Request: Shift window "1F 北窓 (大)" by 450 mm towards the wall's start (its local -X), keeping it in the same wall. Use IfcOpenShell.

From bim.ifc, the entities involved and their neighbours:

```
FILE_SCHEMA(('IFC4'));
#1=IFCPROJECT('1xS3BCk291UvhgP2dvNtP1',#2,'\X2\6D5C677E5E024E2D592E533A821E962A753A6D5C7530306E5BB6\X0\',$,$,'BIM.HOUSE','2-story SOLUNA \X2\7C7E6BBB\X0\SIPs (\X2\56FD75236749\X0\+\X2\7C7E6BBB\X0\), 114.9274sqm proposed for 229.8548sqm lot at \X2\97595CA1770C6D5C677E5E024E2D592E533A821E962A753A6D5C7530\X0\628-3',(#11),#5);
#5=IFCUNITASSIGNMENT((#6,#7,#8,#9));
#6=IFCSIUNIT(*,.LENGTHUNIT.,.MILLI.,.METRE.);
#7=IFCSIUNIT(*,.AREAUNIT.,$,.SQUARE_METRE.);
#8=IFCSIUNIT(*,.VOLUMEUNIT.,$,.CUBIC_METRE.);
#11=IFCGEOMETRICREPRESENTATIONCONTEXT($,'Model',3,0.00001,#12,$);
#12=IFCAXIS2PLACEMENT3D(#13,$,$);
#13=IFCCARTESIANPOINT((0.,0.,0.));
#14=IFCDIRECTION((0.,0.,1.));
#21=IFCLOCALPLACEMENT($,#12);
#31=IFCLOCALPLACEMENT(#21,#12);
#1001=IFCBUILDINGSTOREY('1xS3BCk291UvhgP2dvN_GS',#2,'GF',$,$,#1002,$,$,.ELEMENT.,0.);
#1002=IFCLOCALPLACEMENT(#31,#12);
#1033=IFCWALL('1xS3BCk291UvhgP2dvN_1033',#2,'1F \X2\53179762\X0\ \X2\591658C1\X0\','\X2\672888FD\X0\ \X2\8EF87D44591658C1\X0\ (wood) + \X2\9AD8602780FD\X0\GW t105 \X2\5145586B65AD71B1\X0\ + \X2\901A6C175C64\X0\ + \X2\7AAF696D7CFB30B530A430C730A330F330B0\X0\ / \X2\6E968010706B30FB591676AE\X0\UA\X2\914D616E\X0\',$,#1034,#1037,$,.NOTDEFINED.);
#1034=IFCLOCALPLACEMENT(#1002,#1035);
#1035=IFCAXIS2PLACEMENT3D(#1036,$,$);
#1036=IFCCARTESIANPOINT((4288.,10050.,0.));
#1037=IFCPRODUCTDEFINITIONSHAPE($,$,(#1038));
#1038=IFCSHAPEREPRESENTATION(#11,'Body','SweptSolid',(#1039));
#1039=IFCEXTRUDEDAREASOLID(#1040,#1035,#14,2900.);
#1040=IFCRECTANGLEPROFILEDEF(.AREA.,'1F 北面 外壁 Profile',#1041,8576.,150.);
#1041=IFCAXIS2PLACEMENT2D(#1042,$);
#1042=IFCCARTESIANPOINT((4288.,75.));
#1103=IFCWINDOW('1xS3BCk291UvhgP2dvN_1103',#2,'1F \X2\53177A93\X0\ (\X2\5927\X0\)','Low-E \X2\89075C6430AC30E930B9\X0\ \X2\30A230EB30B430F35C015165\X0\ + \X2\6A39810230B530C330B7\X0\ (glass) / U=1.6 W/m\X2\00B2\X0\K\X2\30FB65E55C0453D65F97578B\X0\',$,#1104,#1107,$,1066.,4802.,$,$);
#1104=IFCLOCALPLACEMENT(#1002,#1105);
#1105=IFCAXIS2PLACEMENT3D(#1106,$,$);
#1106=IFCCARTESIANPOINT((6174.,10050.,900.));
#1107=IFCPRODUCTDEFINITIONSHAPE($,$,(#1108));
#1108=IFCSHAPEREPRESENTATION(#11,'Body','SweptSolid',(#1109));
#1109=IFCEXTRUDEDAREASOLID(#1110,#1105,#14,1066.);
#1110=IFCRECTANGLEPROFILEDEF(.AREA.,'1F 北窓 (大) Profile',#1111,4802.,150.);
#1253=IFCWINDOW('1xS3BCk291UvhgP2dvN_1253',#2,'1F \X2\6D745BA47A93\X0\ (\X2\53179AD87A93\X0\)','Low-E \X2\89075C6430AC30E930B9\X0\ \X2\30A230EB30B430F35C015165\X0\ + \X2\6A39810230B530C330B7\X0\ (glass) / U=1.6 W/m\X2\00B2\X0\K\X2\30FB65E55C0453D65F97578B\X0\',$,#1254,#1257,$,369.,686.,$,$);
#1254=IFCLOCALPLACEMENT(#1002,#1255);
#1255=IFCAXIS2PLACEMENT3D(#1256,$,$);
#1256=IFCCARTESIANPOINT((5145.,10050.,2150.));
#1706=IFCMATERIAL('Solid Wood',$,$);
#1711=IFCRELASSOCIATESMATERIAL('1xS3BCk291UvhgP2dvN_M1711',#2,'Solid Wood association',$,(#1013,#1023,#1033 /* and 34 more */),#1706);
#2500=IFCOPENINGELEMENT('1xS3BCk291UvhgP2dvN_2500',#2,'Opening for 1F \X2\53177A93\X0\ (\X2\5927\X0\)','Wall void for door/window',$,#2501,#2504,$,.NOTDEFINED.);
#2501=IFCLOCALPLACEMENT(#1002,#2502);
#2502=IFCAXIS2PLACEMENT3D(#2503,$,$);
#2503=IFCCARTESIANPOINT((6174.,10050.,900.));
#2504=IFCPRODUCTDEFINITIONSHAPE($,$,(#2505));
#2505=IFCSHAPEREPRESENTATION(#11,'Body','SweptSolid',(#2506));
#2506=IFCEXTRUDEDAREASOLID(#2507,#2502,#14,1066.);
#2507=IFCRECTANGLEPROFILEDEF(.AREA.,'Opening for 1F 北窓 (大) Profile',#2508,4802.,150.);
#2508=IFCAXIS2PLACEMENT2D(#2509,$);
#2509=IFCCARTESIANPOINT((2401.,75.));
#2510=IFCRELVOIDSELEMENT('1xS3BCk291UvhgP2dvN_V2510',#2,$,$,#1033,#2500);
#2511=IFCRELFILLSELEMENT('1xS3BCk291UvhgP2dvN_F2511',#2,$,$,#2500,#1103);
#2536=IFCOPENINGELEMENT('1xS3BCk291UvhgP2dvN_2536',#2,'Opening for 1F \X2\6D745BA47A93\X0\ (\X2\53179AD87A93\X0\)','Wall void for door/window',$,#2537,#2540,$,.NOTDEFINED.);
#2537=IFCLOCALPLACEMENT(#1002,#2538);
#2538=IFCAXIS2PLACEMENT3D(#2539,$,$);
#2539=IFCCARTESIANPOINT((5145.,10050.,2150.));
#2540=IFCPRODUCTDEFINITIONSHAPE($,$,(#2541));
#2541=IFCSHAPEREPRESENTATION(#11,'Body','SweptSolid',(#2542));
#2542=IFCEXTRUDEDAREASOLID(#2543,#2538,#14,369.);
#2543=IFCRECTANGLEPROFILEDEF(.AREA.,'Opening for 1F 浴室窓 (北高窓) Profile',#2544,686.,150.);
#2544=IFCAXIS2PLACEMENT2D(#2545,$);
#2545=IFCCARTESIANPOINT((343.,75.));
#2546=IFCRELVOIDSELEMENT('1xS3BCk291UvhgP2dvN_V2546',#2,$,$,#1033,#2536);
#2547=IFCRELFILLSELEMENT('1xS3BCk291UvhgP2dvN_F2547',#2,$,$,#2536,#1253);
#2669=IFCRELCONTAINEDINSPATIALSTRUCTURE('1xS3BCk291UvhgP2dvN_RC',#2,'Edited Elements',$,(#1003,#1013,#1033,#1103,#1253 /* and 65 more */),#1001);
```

```python
import ifcopenshell
import ifcopenshell.api.geometry
import ifcopenshell.util.placement

model = ifcopenshell.open("bim.ifc")

window = model.by_guid("1xS3BCk291UvhgP2dvN_1103")
opening = window.FillsVoids[0].RelatingOpeningElement
wall = opening.VoidsElements[0].RelatingBuildingElement

wall_matrix = ifcopenshell.util.placement.get_local_placement(wall.ObjectPlacement)
shift = wall_matrix[:3, 0] * -450.0
before = ifcopenshell.util.placement.get_local_placement(window.ObjectPlacement)[:3, 3].copy()

# The window is not placed relative to its opening, so move both.
for product in (opening, window):
    matrix = ifcopenshell.util.placement.get_local_placement(product.ObjectPlacement)
    matrix[:3, 3] += shift
    ifcopenshell.api.geometry.edit_object_placement(model, product=product, matrix=matrix, is_si=False)

after = ifcopenshell.util.placement.get_local_placement(window.ObjectPlacement)[:3, 3]
print("window moved by", (after - before).round(3) + 0.0)

model.write("bim_v2.ifc")
```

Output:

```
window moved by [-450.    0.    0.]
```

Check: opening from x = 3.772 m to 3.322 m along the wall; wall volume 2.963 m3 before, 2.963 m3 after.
